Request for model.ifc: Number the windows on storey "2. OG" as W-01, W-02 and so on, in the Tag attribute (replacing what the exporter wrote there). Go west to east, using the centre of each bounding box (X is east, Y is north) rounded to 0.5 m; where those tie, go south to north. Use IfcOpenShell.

First a look at what the model holds.

```python
import ifcopenshell
import ifcopenshell.util.element
import ifcopenshell.util.placement

model = ifcopenshell.open("model.ifc")
print(model.schema)
storey = next(s for s in model.by_type("IfcBuildingStorey") if s.Name == "2. OG")
windows = [e for e in ifcopenshell.util.element.get_decomposition(storey) if e.is_a("IfcWindow")]
for e in sorted(windows, key=lambda e: e.id()):
    origin = ifcopenshell.util.placement.get_local_placement(e.ObjectPlacement)[:3, 3]
    print(e.id(), e.Tag, e.Name, origin.round(2) + 0.0, sep=" | ")
```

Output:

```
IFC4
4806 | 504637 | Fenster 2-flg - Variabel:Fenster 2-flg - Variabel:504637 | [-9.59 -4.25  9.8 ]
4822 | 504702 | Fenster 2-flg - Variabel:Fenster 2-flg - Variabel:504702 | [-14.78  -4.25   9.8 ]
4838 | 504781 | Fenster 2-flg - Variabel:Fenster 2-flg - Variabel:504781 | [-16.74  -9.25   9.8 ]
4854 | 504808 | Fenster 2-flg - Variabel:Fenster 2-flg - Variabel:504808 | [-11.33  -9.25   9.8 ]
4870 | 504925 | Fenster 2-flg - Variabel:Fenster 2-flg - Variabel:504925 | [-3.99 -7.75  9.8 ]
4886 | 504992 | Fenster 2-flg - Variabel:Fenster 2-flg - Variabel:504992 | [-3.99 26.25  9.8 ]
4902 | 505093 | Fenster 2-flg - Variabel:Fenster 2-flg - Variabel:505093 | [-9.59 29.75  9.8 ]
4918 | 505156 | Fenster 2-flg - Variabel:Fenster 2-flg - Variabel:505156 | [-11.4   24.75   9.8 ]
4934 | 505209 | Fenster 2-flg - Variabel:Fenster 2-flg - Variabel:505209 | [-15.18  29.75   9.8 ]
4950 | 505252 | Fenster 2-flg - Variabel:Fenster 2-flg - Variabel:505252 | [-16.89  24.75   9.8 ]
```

```python
import ifcopenshell
import ifcopenshell.geom
import ifcopenshell.util.element
import ifcopenshell.util.shape

model = ifcopenshell.open("model.ifc")
settings = ifcopenshell.geom.settings()
settings.set("use-world-coords", True)


def centre(element):
    shape = ifcopenshell.geom.create_shape(settings, element)
    return ifcopenshell.util.shape.get_bbox_centroid(shape.geometry)


storey = next(s for s in model.by_type("IfcBuildingStorey") if s.Name == "2. OG")
windows = [e for e in ifcopenshell.util.element.get_decomposition(storey) if e.is_a("IfcWindow")]

# Insertion points can sit at a corner or the storey origin, so sort by the geometry (in metres).
centres = {e: centre(e) for e in windows}
windows.sort(key=lambda e: (round(centres[e][0] / 0.5), centres[e][1]))

for i, e in enumerate(windows, start=1):
    number = f"W-{i:02d}"
    e.Tag = number
    print(e.id(), number)

model.write("model-out.ifc")
```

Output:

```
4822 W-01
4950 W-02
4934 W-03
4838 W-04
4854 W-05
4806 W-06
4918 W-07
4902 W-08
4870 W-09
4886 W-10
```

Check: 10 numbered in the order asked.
